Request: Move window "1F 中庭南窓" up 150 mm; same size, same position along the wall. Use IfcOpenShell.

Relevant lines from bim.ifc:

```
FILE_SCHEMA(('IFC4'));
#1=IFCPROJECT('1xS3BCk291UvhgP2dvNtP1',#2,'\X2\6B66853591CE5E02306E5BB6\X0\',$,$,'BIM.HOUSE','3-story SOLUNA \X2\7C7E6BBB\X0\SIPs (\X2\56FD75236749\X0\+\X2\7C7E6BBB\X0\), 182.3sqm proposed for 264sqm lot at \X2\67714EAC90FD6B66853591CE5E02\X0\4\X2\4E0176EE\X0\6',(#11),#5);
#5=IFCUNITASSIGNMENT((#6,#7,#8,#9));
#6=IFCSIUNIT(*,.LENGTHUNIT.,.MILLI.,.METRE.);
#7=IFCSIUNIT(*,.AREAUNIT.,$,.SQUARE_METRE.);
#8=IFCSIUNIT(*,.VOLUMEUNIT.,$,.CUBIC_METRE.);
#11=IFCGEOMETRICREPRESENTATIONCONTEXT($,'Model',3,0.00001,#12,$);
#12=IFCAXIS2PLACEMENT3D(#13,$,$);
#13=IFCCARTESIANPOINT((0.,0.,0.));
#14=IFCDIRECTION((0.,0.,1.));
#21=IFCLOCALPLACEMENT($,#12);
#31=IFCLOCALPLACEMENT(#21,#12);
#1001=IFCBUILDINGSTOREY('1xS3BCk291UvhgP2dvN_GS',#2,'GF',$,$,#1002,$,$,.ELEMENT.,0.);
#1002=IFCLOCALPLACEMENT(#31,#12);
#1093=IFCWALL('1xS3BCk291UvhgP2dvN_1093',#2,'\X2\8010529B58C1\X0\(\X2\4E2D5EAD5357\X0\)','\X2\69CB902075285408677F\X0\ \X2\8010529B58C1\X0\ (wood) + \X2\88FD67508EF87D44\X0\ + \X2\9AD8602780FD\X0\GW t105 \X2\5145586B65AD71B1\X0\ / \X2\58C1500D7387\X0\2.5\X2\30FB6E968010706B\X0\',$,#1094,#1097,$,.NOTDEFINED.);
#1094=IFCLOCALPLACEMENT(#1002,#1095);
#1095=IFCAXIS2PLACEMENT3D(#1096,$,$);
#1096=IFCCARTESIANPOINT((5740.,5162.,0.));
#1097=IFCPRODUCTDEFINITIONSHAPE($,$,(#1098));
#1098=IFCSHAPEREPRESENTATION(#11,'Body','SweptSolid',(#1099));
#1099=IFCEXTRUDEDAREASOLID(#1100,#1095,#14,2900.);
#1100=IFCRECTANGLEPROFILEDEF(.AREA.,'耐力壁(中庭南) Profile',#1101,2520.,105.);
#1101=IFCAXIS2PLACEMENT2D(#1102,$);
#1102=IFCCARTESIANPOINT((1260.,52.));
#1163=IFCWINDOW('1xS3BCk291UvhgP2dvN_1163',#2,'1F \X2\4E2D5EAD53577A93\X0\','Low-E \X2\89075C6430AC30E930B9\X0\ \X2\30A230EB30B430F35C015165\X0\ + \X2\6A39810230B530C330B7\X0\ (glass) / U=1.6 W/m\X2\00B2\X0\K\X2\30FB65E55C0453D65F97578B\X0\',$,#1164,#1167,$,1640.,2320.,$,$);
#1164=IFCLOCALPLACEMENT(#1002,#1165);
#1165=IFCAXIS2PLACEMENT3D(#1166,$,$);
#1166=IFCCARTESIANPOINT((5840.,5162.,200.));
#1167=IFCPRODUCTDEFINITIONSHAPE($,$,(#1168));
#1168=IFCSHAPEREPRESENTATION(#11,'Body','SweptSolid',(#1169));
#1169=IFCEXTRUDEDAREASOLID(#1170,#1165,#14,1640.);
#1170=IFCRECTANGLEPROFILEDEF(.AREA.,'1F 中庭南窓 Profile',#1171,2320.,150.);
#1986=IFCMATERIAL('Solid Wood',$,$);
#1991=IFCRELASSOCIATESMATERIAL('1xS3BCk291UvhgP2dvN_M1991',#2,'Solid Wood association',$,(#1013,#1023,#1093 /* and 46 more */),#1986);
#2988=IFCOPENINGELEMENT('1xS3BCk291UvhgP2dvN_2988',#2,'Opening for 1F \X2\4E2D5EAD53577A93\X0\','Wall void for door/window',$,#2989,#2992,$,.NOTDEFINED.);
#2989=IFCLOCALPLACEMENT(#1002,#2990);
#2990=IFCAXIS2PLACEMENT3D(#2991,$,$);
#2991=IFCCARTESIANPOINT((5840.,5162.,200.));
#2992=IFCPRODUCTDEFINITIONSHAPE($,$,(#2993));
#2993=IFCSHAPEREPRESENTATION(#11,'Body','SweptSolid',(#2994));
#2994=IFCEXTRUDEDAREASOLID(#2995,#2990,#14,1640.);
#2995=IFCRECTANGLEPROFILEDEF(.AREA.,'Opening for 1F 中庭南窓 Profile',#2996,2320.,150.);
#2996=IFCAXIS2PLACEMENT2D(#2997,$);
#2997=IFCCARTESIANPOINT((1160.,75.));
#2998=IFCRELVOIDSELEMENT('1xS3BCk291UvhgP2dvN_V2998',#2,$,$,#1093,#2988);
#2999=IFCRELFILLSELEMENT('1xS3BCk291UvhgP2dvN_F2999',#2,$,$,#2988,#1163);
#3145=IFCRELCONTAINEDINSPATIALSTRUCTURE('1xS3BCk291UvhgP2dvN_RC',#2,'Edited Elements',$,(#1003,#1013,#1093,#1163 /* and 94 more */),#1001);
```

```python
import numpy as np
import ifcopenshell
import ifcopenshell.api.geometry
import ifcopenshell.util.placement
import ifcopenshell.util.unit

model = ifcopenshell.open("bim.ifc")
unit_scale = ifcopenshell.util.unit.calculate_unit_scale(model)

window = model.by_guid("1xS3BCk291UvhgP2dvN_1163")
opening = window.FillsVoids[0].RelatingOpeningElement
dz = 0.15 / unit_scale

shift = np.array([0.0, 0.0, dz])
# The window is not placed relative to its opening, so move both.
for product in (opening, window):
    matrix = ifcopenshell.util.placement.get_local_placement(product.ObjectPlacement)
    matrix[:3, 3] += shift
    ifcopenshell.api.geometry.edit_object_placement(model, product=product, matrix=matrix, is_si=False)

print(f"moved by {dz * unit_scale:+.3f} m")

model.write("bim_edited.ifc")
```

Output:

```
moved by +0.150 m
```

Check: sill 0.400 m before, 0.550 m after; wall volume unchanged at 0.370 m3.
